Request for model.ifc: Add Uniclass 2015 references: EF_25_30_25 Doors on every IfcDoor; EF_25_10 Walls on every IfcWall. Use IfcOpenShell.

First a look at what the model holds.

```python
import ifcopenshell

model = ifcopenshell.open("model.ifc")
print(model.schema)
print("classifications:", [c.Name for c in model.by_type("IfcClassification")])
for ifc_class in ("IfcDoor", "IfcRoof", "IfcStair", "IfcWall", "IfcWindow"):
    print(ifc_class, len(model.by_type(ifc_class)))
```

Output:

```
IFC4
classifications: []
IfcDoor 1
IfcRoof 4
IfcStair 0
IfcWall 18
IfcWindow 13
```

```python
import ifcopenshell
import ifcopenshell.api.classification

model = ifcopenshell.open("model.ifc")

system = ifcopenshell.api.classification.add_classification(model, classification="Uniclass 2015")

codes = {
    "IfcDoor": ("EF_25_30_25", "Doors"),
    "IfcWall": ("EF_25_10", "Walls"),
}
for ifc_class, (code, name) in codes.items():
    products = model.by_type(ifc_class)
    ifcopenshell.api.classification.add_reference(
        model, products=products, classification=system, identification=code, name=name
    )
    print(code, len(products))

model.write("model_rev.ifc")
```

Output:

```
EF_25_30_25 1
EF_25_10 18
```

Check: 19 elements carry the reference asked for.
